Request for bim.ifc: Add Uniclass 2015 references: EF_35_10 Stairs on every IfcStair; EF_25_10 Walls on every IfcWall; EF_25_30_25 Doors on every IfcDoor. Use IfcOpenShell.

First a look at what the model holds.

```python
import ifcopenshell

model = ifcopenshell.open("bim.ifc")
print(model.schema)
print("classifications:", [c.Name for c in model.by_type("IfcClassification")])
for ifc_class in ("IfcDoor", "IfcRoof", "IfcStair", "IfcWall", "IfcWindow"):
    print(ifc_class, len(model.by_type(ifc_class)))
```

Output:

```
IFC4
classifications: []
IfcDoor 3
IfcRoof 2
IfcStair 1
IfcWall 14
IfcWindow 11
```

```python
import ifcopenshell
import ifcopenshell.api.classification

model = ifcopenshell.open("bim.ifc")

system = ifcopenshell.api.classification.add_classification(model, classification="Uniclass 2015")

codes = {
    "IfcStair": ("EF_35_10", "Stairs"),
    "IfcWall": ("EF_25_10", "Walls"),
    "IfcDoor": ("EF_25_30_25", "Doors"),
}
for ifc_class, (code, name) in codes.items():
    products = model.by_type(ifc_class)
    ifcopenshell.api.classification.add_reference(
        model, products=products, classification=system, identification=code, name=name
    )
    print(code, len(products))

model.write("bim-out.ifc")
```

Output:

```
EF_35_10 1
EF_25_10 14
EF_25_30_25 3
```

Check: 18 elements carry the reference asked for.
